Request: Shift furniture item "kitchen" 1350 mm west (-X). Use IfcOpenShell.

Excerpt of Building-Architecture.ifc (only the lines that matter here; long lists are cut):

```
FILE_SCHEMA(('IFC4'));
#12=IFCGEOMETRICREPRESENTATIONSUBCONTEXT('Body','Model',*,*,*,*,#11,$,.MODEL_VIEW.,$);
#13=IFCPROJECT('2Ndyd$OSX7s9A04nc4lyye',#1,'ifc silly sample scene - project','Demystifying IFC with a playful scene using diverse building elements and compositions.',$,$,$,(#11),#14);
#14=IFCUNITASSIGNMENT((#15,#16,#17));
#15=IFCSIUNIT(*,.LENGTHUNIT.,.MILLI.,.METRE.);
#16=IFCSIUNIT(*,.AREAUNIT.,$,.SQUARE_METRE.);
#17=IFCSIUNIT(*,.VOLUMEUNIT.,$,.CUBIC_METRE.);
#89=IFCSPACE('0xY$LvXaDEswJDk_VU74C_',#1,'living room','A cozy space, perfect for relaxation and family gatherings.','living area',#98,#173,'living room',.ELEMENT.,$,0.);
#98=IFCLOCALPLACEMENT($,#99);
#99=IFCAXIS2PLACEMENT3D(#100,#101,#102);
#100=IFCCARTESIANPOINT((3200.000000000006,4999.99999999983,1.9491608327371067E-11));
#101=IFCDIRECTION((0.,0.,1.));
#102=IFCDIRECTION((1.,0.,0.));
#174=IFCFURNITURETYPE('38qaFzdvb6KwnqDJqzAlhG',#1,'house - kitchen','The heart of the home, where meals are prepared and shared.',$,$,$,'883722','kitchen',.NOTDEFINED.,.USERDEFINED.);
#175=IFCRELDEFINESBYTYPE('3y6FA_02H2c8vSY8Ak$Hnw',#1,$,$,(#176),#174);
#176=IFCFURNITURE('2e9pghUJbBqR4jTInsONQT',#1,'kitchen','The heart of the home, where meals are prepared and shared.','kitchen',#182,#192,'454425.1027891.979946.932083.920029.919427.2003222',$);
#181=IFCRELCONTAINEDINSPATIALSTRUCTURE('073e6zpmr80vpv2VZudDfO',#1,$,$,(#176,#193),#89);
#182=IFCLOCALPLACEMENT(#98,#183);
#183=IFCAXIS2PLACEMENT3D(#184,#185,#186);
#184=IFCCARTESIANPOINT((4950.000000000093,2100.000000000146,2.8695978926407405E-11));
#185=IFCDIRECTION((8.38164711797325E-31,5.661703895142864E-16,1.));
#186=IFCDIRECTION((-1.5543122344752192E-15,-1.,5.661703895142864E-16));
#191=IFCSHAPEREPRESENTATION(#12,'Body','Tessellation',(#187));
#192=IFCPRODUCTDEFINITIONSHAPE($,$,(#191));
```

```python
import ifcopenshell
import ifcopenshell.api.geometry
import ifcopenshell.util.placement
import ifcopenshell.util.unit

model = ifcopenshell.open("Building-Architecture.ifc")
unit_scale = ifcopenshell.util.unit.calculate_unit_scale(model)

item = model.by_guid("2e9pghUJbBqR4jTInsONQT")
matrix = ifcopenshell.util.placement.get_local_placement(item.ObjectPlacement)
matrix[0, 3] -= 1.35 / unit_scale
ifcopenshell.api.geometry.edit_object_placement(model, product=item, matrix=matrix, is_si=False)

print(ifcopenshell.util.placement.get_local_placement(item.ObjectPlacement).round(3) + 0.0)

model.write("Building-Architecture_updated.ifc")
```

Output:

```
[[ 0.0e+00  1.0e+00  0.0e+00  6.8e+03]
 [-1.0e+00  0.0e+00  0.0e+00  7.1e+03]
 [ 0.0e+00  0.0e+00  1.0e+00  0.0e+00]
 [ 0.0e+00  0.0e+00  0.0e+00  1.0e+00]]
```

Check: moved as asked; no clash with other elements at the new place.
